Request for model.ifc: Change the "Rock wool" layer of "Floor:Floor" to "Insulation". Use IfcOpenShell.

First a look at what the model holds.

```python
import ifcopenshell
import ifcopenshell.util.element

model = ifcopenshell.open("model.ifc")
print(model.schema)
for layer_set in model.by_type("IfcMaterialLayerSet"):
    if layer_set.LayerSetName == "Floor:Floor":
        for layer in layer_set.MaterialLayers:
            print(layer.id(), layer.Material and layer.Material.Name, layer.LayerThickness, sep=" | ")
        print(len(ifcopenshell.util.element.get_elements_by_material(model, layer_set)), "elements and types use it")
print(sorted(m.Name for m in model.by_type("IfcMaterial") if m.Name)[:60])
```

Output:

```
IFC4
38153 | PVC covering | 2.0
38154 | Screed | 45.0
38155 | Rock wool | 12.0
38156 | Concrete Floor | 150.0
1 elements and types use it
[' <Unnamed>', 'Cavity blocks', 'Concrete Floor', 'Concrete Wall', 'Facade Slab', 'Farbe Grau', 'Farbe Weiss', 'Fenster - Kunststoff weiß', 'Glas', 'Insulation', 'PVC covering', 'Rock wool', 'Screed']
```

```python
import ifcopenshell
import ifcopenshell.api.material

model = ifcopenshell.open("model.ifc")

layer_set = next(s for s in model.by_type("IfcMaterialLayerSet") if s.LayerSetName == "Floor:Floor")
layer = next(l for l in layer_set.MaterialLayers if l.Material and l.Material.Name == "Rock wool")
material = next(m for m in model.by_type("IfcMaterial") if m.Name == "Insulation")

# Point this one layer at the other material; renaming the old one would change it everywhere.
ifcopenshell.api.material.edit_layer(model, layer=layer, attributes={}, material=material)

print([l.Material.Name if l.Material else None for l in layer_set.MaterialLayers])

model.write("model_edited.ifc")
```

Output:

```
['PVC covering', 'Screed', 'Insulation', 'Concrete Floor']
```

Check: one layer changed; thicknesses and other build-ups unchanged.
